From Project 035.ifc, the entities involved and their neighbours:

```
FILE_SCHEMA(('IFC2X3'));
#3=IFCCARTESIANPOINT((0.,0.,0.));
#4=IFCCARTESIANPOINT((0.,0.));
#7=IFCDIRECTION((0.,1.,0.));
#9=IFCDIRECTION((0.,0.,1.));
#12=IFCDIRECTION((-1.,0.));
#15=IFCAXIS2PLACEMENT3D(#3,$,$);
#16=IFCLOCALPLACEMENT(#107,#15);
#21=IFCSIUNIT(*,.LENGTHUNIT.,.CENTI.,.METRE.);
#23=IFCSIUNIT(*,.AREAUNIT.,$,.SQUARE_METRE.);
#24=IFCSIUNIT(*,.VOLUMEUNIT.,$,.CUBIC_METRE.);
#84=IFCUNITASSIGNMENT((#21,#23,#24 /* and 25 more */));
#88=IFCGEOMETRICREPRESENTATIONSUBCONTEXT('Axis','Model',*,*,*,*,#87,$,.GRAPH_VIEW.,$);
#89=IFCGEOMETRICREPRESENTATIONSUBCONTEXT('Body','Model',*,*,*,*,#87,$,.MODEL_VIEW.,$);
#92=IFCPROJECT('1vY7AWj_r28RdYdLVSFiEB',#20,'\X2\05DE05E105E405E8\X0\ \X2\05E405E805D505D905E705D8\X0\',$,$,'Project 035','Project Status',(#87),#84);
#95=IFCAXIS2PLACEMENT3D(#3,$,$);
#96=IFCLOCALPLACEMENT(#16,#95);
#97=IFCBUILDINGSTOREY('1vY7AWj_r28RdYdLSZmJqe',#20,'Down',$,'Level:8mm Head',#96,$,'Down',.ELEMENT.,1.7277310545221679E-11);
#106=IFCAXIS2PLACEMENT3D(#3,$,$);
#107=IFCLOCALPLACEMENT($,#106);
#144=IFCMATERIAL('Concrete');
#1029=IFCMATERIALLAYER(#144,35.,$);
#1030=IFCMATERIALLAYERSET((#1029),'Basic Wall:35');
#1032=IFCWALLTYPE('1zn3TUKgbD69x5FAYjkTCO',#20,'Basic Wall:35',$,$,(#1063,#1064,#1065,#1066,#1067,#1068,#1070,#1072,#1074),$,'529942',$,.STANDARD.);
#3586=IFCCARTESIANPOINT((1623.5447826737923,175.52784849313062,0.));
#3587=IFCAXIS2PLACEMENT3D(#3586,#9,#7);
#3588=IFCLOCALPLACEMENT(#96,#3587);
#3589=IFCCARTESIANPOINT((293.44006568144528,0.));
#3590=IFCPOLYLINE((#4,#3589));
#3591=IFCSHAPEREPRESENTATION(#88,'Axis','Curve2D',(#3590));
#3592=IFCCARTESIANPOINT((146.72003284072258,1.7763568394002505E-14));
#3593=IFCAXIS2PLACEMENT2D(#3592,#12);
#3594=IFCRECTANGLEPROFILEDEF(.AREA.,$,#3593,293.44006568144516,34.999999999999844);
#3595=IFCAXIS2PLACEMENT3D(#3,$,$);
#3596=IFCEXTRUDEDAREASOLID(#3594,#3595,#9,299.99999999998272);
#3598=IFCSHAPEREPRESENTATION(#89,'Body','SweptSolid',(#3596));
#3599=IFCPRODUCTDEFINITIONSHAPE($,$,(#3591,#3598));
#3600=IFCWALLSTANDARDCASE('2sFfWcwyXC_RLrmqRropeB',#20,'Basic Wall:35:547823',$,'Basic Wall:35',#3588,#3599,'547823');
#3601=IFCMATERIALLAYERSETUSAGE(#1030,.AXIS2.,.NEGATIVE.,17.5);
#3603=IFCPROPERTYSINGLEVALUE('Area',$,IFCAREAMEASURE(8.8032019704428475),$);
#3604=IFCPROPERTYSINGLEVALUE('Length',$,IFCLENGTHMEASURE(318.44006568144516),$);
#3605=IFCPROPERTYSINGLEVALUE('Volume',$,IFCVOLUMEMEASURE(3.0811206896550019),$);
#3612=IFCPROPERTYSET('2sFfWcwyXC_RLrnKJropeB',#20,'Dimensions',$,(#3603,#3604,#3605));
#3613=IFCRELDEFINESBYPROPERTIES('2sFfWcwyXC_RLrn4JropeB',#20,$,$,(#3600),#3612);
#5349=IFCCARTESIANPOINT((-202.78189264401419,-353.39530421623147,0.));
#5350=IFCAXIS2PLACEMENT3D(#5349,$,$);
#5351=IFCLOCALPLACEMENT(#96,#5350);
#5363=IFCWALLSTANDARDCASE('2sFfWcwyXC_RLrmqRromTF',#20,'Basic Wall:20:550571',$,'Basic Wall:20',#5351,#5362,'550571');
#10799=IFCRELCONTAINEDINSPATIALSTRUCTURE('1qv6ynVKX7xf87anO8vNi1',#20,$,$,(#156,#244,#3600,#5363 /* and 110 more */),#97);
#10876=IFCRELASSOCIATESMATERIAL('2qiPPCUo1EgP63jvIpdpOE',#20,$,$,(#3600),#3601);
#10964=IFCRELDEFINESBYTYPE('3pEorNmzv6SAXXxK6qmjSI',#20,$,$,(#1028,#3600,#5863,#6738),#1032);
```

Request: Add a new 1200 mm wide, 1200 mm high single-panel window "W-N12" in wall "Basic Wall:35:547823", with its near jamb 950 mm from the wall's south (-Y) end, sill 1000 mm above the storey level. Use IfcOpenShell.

```python
import numpy as np
import ifcopenshell
import ifcopenshell.api.feature
import ifcopenshell.api.geometry
import ifcopenshell.api.pset
import ifcopenshell.api.root
import ifcopenshell.api.spatial
import ifcopenshell.api.type
import ifcopenshell.geom
import ifcopenshell.util.element
import ifcopenshell.util.placement
import ifcopenshell.util.representation
import ifcopenshell.util.shape
import ifcopenshell.util.unit

model = ifcopenshell.open("Project 035.ifc")
unit_scale = ifcopenshell.util.unit.calculate_unit_scale(model)
area_scale = ifcopenshell.util.unit.calculate_unit_scale(model, "AREAUNIT")
volume_scale = ifcopenshell.util.unit.calculate_unit_scale(model, "VOLUMEUNIT")
settings = ifcopenshell.geom.settings()


def volume(element):
    """Net volume in cubic metres, openings subtracted."""
    shape = ifcopenshell.geom.create_shape(settings, element)
    return ifcopenshell.util.shape.get_volume(shape.geometry)


wall = model.by_guid("2sFfWcwyXC_RLrmqRropeB")
storey = ifcopenshell.util.element.get_container(wall, ifc_class="IfcBuildingStorey")
context = ifcopenshell.util.representation.get_context(model, "Model", "Body", "MODEL_VIEW")
before = volume(wall)

width, height, from_end, sill = 1.2, 1.2, 0.95, 1  # metres

# The wall runs along its own X axis, and the end named is its -X end.
wall_shape = ifcopenshell.geom.create_shape(settings, wall)
x, y, z = ifcopenshell.util.shape.get_vertices(wall_shape.geometry).T
start = x.min() + from_end
face, thickness = float(y.min()), float(y.max() - y.min())
wall_matrix = ifcopenshell.util.placement.get_local_placement(wall.ObjectPlacement)
level = ifcopenshell.util.placement.get_local_placement(storey.ObjectPlacement)[2, 3]


def in_wall(x, y):
    """Placement at x, y metres in the wall's axes, at sill height."""
    matrix = wall_matrix.copy()
    matrix[:, 3] = wall_matrix @ np.array([x / unit_scale, y / unit_scale, 0.0, 1.0])
    matrix[2, 3] = level + sill / unit_scale
    return matrix


# Opening: a box that overshoots both wall faces by 50 mm.
opening = ifcopenshell.api.root.create_entity(model, ifc_class="IfcOpeningElement")
box = ifcopenshell.api.geometry.add_wall_representation(
    model, context=context, length=width, height=height, thickness=thickness + 0.1
)
ifcopenshell.api.geometry.assign_representation(model, product=opening, representation=box)
ifcopenshell.api.geometry.edit_object_placement(model, product=opening, matrix=in_wall(start, face - 0.05), is_si=False)
ifcopenshell.api.feature.add_feature(model, feature=opening, element=wall)

window = ifcopenshell.api.root.create_entity(model, ifc_class="IfcWindow", name="W-N12")
window.OverallWidth, window.OverallHeight = width / unit_scale, height / unit_scale
body = ifcopenshell.api.geometry.add_window_representation(
    model,
    context=context,
    overall_width=window.OverallWidth,
    overall_height=window.OverallHeight,
    partition_type="SINGLE_PANEL",
)
ifcopenshell.api.geometry.assign_representation(model, product=window, representation=body)
ifcopenshell.api.spatial.assign_container(model, products=[window], relating_structure=storey)
fills = ifcopenshell.api.feature.add_filling(model, opening=opening, element=window)
fills.OwnerHistory = window.OwnerHistory  # required in IFC2X3

# IFC2X3 keeps the operation on the window style.
style = ifcopenshell.api.root.create_entity(model, ifc_class="IfcWindowStyle", name="W-N12")
style.OperationType, style.ConstructionType = "SINGLE_PANEL", "NOTDEFINED"
style.ParameterTakesPrecedence = style.Sizeable = False
ifcopenshell.api.type.assign_type(model, related_objects=[window], relating_type=style)

# Centre the window in the wall's thickness.
ifcopenshell.api.geometry.edit_object_placement(model, product=window, matrix=in_wall(start, face), is_si=False)
window_shape = ifcopenshell.geom.create_shape(settings, window)
depth = ifcopenshell.util.shape.get_vertices(window_shape.geometry)[:, 1]
offset = face + thickness / 2 - (depth.min() + depth.max()) / 2
ifcopenshell.api.geometry.edit_object_placement(model, product=window, matrix=in_wall(start, offset), is_si=False)

after = volume(wall)

# Update the wall's stored quantities.
pset = model.by_id(ifcopenshell.util.element.get_pset(wall, "Dimensions", should_inherit=False)["id"])
ifcopenshell.api.pset.edit_pset(model, pset=pset, properties={
    "Area": model.create_entity("IfcAreaMeasure", after / thickness / area_scale),
    "Volume": model.create_entity("IfcVolumeMeasure", after / volume_scale),
})

print(f"wall volume {before:.3f} -> {after:.3f} m3")

model.write("Project 035_rev.ifc")
```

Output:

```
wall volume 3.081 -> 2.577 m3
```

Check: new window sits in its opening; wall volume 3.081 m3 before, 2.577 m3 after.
